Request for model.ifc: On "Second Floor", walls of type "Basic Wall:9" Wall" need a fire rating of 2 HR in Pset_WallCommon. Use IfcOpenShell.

First a look at what the model holds.

```python
import ifcopenshell
import ifcopenshell.util.element

model = ifcopenshell.open("model.ifc")
print(model.schema)
storey = next(s for s in model.by_type("IfcBuildingStorey") if s.Name == "Second Floor")
walls = [e for e in ifcopenshell.util.element.get_decomposition(storey) if e.is_a("IfcWall")]
seen = {}
for e in walls:
    element_type = ifcopenshell.util.element.get_type(e)
    key = (element_type.Name if element_type != e and element_type else None, ifcopenshell.util.element.get_pset(e, "Pset_WallCommon", "FireRating"))
    seen[key] = seen.get(key, 0) + 1
for (name, value), count in sorted(seen.items(), key=str):
    print(count, "x", name, "|", value)
```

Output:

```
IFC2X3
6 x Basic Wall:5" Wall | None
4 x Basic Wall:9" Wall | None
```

```python
import ifcopenshell
import ifcopenshell.api.pset
import ifcopenshell.util.element

model = ifcopenshell.open("model.ifc")

storey = next(s for s in model.by_type("IfcBuildingStorey") if s.Name == "Second Floor")
walls = [e for e in ifcopenshell.util.element.get_decomposition(storey) if e.is_a("IfcWall")]

count = 0
for e in walls:
    element_type = ifcopenshell.util.element.get_type(e)
    if element_type in (None, e) or element_type.Name != 'Basic Wall:9" Wall':
        continue
    # add_pset returns the element's existing set when there is one.
    pset = ifcopenshell.api.pset.add_pset(model, product=e, name="Pset_WallCommon")
    ifcopenshell.api.pset.edit_pset(model, pset=pset, properties={"FireRating": "2 HR"})
    count += 1

print(count, "walls updated")

model.write("model_v2.ifc")
```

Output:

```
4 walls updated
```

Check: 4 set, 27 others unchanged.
